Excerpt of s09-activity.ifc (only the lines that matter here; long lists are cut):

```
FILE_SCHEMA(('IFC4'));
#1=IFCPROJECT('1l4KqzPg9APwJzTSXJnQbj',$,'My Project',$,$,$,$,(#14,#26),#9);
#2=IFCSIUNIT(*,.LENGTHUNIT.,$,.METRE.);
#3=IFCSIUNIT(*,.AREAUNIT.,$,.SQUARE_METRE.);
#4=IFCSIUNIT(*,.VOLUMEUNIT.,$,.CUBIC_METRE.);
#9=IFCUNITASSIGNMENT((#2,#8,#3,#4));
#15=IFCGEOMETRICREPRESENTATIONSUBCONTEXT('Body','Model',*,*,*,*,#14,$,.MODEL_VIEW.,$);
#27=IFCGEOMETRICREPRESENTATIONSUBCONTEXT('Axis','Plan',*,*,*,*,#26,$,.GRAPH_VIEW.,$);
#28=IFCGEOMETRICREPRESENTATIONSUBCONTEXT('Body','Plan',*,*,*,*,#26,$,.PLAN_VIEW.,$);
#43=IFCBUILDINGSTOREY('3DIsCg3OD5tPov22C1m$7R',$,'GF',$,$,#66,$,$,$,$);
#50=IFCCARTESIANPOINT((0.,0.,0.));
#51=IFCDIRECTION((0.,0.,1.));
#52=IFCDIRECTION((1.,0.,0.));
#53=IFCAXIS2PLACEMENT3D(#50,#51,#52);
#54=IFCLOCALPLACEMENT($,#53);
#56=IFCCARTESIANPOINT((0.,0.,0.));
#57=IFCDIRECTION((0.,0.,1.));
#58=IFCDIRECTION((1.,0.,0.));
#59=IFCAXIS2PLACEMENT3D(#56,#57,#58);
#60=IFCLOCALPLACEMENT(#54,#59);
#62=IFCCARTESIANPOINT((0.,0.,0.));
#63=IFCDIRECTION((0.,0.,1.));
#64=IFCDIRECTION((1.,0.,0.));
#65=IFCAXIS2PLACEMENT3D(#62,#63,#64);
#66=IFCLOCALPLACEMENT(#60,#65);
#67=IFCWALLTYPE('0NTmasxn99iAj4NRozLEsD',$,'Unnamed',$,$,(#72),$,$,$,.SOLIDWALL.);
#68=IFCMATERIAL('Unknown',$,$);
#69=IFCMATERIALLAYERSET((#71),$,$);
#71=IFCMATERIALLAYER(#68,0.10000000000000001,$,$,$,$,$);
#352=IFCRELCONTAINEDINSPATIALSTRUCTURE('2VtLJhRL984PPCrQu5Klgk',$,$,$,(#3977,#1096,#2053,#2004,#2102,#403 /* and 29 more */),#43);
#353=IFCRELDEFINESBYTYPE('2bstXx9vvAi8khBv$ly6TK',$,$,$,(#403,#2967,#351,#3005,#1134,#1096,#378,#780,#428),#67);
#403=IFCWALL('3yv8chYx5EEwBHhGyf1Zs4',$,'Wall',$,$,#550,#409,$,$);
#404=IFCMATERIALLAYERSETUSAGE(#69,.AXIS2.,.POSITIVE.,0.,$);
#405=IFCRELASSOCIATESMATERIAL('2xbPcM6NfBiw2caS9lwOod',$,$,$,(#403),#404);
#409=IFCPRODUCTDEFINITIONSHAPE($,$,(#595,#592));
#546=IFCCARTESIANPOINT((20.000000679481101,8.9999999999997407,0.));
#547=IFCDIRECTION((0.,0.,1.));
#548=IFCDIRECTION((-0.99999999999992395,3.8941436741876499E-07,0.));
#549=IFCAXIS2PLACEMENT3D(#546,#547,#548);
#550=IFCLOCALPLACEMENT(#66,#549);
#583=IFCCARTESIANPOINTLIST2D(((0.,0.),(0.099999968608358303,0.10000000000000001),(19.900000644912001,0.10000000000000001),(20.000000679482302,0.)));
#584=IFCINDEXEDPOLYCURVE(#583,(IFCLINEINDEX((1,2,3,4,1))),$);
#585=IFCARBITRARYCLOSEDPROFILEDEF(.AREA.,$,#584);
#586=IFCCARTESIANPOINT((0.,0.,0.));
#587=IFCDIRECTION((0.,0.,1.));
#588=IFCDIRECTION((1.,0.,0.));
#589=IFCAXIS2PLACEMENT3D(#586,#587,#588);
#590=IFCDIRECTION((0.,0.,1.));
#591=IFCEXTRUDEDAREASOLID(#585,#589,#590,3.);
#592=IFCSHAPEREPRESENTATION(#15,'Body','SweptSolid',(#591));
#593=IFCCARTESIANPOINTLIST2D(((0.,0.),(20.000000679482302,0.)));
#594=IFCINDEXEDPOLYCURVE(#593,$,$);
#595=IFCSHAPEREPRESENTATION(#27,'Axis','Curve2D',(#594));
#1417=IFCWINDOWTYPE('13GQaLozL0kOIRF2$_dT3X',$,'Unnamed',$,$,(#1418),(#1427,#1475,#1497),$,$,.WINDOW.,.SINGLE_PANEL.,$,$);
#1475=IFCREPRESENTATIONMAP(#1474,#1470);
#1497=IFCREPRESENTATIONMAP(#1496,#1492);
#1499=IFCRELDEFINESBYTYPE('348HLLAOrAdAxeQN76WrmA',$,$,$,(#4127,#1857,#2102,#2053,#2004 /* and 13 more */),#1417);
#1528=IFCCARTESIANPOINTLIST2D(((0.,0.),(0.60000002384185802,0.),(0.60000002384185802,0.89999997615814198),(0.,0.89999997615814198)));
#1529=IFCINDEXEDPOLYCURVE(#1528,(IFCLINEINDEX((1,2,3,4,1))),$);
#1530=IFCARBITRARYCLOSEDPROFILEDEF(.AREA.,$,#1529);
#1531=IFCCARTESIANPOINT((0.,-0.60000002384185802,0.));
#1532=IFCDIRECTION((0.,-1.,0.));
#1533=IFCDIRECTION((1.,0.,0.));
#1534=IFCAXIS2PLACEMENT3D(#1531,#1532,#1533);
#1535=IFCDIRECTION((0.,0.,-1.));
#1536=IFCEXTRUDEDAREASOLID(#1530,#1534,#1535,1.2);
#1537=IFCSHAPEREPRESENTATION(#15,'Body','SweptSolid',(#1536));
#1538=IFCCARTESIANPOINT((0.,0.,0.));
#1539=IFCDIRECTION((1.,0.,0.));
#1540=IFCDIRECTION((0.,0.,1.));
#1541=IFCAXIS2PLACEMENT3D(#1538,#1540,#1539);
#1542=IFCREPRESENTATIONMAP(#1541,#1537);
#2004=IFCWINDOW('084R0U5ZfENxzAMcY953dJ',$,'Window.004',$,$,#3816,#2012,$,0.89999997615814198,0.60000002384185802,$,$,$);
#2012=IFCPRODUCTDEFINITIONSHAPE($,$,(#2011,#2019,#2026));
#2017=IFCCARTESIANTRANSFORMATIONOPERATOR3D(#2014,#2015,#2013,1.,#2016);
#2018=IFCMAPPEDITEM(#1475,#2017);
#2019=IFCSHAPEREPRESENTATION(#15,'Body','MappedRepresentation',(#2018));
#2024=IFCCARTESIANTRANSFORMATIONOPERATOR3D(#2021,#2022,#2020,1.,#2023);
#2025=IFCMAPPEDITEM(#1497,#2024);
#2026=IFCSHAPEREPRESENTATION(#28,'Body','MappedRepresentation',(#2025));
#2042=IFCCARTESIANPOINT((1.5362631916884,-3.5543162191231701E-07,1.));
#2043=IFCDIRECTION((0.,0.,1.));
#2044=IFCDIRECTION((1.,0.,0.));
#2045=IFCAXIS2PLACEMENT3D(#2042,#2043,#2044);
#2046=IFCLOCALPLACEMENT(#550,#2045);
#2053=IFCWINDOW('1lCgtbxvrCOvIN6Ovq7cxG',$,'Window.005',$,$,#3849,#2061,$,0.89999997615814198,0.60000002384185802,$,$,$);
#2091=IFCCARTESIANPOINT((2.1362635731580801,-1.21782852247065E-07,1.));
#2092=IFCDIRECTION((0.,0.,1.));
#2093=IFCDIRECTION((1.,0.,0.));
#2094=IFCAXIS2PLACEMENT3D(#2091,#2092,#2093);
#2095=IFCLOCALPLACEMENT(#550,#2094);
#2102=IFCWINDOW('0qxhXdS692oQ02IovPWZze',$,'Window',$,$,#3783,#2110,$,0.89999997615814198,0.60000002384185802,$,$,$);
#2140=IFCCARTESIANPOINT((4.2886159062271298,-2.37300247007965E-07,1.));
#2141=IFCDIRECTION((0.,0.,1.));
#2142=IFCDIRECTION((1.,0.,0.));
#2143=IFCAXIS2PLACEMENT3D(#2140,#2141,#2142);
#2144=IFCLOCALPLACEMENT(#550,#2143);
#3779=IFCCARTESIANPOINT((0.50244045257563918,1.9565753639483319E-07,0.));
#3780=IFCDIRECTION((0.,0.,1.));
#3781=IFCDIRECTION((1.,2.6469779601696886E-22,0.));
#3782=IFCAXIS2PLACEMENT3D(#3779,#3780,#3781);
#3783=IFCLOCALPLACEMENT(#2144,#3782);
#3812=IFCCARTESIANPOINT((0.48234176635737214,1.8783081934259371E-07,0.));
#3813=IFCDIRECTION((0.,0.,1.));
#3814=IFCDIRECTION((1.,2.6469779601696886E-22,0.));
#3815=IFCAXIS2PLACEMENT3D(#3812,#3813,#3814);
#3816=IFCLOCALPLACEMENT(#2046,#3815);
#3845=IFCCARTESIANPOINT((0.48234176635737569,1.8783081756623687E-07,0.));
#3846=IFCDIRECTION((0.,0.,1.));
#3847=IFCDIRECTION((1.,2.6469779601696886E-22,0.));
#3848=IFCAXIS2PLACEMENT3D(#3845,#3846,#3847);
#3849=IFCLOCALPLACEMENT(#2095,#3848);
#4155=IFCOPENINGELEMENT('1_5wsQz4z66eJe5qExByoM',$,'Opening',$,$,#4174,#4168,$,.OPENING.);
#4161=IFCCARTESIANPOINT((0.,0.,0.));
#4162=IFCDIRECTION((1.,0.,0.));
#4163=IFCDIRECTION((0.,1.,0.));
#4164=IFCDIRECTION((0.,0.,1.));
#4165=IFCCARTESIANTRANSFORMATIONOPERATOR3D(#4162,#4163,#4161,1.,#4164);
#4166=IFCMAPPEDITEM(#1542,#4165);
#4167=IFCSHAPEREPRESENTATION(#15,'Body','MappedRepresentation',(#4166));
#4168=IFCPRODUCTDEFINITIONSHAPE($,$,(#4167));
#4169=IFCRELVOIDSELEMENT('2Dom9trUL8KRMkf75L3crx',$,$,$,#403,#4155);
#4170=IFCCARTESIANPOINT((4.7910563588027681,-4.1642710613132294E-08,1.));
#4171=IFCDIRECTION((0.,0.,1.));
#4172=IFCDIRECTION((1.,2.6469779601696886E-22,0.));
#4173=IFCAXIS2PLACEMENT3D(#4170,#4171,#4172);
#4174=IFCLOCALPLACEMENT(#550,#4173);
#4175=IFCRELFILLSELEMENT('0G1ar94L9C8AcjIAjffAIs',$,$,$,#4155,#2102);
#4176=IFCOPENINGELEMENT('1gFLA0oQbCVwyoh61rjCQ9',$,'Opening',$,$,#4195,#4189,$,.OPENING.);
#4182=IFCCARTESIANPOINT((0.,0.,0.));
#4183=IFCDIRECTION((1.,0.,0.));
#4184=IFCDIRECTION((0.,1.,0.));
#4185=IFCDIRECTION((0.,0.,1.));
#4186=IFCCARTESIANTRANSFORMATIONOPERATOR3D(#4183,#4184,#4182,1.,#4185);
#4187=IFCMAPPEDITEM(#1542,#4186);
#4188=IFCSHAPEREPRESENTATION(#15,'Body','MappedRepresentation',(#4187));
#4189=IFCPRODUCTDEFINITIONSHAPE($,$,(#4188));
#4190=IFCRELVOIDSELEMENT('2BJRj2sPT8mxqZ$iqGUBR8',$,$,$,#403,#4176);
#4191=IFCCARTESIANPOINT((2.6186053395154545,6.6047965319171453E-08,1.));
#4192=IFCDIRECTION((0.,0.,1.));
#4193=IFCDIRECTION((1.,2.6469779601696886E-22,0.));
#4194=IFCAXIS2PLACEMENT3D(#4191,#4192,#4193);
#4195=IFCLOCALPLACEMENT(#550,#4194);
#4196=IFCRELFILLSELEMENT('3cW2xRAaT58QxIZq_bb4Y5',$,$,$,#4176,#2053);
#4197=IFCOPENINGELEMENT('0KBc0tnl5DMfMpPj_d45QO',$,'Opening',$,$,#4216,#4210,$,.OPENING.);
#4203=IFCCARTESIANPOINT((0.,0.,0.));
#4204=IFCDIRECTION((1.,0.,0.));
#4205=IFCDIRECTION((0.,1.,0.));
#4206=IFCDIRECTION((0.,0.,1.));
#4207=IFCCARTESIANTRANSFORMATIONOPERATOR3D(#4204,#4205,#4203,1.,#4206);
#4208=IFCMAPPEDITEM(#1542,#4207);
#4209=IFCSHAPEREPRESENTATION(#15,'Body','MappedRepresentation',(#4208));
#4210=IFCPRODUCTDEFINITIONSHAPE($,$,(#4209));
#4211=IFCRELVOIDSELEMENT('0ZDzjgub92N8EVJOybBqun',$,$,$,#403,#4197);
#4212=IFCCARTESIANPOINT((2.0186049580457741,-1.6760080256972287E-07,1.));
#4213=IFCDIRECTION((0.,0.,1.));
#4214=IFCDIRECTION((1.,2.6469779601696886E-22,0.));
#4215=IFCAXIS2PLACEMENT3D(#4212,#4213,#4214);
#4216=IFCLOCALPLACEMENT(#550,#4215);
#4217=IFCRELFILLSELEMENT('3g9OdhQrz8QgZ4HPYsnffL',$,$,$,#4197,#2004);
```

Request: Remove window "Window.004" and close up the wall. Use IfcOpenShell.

```python
import ifcopenshell
import ifcopenshell.api.feature
import ifcopenshell.api.root
import ifcopenshell.geom
import ifcopenshell.util.shape

model = ifcopenshell.open("s09-activity.ifc")
settings = ifcopenshell.geom.settings()


def volume(element):
    """Net volume in cubic metres, openings subtracted."""
    shape = ifcopenshell.geom.create_shape(settings, element)
    return ifcopenshell.util.shape.get_volume(shape.geometry)


window = model.by_guid("084R0U5ZfENxzAMcY953dJ")
opening = window.FillsVoids[0].RelatingOpeningElement
wall = opening.VoidsElements[0].RelatingBuildingElement
before = volume(wall)

ifcopenshell.api.root.remove_product(model, product=window)
ifcopenshell.api.feature.remove_feature(model, feature=opening)

after = volume(wall)

print(f"wall volume {before:.3f} -> {after:.3f} m3")

model.write("s09-activity_rev.ifc")
```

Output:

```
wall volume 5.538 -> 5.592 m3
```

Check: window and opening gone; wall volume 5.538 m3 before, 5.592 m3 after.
